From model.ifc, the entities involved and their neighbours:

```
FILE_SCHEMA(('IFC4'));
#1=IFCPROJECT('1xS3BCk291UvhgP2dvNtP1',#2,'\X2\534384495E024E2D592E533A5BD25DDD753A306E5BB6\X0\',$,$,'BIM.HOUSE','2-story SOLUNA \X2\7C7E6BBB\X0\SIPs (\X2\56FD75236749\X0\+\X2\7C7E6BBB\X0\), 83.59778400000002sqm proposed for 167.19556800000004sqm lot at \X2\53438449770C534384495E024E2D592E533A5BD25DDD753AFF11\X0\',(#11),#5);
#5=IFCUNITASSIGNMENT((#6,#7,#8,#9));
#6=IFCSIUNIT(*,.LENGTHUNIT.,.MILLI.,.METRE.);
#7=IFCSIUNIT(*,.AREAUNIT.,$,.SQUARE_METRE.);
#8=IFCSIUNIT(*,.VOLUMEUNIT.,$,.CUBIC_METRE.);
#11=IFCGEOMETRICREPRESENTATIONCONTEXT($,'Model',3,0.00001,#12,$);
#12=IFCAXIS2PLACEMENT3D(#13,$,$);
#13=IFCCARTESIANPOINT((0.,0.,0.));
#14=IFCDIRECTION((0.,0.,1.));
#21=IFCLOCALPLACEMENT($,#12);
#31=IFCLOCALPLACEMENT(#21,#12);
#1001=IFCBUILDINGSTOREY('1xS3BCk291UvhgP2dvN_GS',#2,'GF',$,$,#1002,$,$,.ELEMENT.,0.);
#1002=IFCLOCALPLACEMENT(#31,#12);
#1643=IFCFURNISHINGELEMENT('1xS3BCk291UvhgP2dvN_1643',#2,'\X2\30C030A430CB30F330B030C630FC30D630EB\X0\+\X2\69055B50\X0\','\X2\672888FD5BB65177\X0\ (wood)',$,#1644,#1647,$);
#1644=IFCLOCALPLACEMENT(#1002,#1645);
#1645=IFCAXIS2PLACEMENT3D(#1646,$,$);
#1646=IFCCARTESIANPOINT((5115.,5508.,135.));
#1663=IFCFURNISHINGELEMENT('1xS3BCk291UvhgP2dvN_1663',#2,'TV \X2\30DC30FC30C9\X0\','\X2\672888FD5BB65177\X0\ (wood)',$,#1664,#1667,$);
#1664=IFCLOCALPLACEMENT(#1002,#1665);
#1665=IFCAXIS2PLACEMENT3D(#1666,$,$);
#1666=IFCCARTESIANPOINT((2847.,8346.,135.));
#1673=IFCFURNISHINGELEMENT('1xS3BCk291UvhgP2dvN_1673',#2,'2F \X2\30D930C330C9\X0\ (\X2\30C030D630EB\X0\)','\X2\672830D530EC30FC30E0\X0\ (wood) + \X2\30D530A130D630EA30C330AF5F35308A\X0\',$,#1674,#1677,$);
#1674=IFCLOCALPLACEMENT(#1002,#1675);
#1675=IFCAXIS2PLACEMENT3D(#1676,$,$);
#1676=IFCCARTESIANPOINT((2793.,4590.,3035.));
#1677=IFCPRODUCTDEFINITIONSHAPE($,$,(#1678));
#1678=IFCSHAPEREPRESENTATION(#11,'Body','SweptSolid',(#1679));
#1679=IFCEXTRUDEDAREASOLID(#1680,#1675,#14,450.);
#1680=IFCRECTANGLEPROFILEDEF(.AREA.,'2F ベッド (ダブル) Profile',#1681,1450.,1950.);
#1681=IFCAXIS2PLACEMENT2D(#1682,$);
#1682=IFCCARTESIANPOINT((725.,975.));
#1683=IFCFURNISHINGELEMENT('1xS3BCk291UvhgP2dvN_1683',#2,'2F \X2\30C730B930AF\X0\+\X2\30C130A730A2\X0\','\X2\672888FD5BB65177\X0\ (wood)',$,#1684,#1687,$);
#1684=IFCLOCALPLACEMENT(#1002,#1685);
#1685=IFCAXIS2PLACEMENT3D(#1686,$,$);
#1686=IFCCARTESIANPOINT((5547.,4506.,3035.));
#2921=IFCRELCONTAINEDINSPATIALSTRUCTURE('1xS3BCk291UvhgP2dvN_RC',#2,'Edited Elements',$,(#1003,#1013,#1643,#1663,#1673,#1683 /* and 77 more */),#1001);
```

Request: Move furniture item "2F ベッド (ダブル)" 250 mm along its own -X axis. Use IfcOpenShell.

```python
import ifcopenshell
import ifcopenshell.api.geometry
import ifcopenshell.util.placement

model = ifcopenshell.open("model.ifc")

item = model.by_id(1673)
matrix = ifcopenshell.util.placement.get_local_placement(item.ObjectPlacement)
matrix[:3, 3] -= matrix[:3, 0] * 250.0
ifcopenshell.api.geometry.edit_object_placement(model, product=item, matrix=matrix, is_si=False)

print(ifcopenshell.util.placement.get_local_placement(item.ObjectPlacement).round(3) + 0.0)

model.write("model_rev.ifc")
```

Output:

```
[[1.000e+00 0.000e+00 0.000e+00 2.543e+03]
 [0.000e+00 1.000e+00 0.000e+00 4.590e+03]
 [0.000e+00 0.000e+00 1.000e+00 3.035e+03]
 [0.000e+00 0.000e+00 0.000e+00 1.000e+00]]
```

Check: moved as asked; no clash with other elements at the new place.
